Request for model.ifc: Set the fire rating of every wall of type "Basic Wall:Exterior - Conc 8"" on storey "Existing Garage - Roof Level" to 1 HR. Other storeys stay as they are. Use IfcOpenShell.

First a look at what the model holds.

```python
import ifcopenshell
import ifcopenshell.util.element

model = ifcopenshell.open("model.ifc")
print(model.schema)
storey = next(s for s in model.by_type("IfcBuildingStorey") if s.Name == "Existing Garage - Roof Level")
walls = [e for e in ifcopenshell.util.element.get_decomposition(storey) if e.is_a("IfcWall")]
seen = {}
for e in walls:
    element_type = ifcopenshell.util.element.get_type(e)
    key = (element_type.Name if element_type != e and element_type else None, ifcopenshell.util.element.get_pset(e, "Pset_WallCommon", "FireRating"))
    seen[key] = seen.get(key, 0) + 1
for (name, value), count in sorted(seen.items(), key=str):
    print(count, "x", name, "|", value)
```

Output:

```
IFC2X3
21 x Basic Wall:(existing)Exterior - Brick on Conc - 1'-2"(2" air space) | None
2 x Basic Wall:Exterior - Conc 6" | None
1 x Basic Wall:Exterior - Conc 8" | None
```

```python
import ifcopenshell
import ifcopenshell.api.pset
import ifcopenshell.util.element

model = ifcopenshell.open("model.ifc")

storey = next(s for s in model.by_type("IfcBuildingStorey") if s.Name == "Existing Garage - Roof Level")
walls = [e for e in ifcopenshell.util.element.get_decomposition(storey) if e.is_a("IfcWall")]

count = 0
for e in walls:
    element_type = ifcopenshell.util.element.get_type(e)
    if element_type in (None, e) or element_type.Name != 'Basic Wall:Exterior - Conc 8"':
        continue
    # add_pset returns the element's existing set when there is one.
    pset = ifcopenshell.api.pset.add_pset(model, product=e, name="Pset_WallCommon")
    ifcopenshell.api.pset.edit_pset(model, pset=pset, properties={"FireRating": "1 HR"})
    count += 1

print(count, "walls updated")

model.write("model_updated.ifc")
```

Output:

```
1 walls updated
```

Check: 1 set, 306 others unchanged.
